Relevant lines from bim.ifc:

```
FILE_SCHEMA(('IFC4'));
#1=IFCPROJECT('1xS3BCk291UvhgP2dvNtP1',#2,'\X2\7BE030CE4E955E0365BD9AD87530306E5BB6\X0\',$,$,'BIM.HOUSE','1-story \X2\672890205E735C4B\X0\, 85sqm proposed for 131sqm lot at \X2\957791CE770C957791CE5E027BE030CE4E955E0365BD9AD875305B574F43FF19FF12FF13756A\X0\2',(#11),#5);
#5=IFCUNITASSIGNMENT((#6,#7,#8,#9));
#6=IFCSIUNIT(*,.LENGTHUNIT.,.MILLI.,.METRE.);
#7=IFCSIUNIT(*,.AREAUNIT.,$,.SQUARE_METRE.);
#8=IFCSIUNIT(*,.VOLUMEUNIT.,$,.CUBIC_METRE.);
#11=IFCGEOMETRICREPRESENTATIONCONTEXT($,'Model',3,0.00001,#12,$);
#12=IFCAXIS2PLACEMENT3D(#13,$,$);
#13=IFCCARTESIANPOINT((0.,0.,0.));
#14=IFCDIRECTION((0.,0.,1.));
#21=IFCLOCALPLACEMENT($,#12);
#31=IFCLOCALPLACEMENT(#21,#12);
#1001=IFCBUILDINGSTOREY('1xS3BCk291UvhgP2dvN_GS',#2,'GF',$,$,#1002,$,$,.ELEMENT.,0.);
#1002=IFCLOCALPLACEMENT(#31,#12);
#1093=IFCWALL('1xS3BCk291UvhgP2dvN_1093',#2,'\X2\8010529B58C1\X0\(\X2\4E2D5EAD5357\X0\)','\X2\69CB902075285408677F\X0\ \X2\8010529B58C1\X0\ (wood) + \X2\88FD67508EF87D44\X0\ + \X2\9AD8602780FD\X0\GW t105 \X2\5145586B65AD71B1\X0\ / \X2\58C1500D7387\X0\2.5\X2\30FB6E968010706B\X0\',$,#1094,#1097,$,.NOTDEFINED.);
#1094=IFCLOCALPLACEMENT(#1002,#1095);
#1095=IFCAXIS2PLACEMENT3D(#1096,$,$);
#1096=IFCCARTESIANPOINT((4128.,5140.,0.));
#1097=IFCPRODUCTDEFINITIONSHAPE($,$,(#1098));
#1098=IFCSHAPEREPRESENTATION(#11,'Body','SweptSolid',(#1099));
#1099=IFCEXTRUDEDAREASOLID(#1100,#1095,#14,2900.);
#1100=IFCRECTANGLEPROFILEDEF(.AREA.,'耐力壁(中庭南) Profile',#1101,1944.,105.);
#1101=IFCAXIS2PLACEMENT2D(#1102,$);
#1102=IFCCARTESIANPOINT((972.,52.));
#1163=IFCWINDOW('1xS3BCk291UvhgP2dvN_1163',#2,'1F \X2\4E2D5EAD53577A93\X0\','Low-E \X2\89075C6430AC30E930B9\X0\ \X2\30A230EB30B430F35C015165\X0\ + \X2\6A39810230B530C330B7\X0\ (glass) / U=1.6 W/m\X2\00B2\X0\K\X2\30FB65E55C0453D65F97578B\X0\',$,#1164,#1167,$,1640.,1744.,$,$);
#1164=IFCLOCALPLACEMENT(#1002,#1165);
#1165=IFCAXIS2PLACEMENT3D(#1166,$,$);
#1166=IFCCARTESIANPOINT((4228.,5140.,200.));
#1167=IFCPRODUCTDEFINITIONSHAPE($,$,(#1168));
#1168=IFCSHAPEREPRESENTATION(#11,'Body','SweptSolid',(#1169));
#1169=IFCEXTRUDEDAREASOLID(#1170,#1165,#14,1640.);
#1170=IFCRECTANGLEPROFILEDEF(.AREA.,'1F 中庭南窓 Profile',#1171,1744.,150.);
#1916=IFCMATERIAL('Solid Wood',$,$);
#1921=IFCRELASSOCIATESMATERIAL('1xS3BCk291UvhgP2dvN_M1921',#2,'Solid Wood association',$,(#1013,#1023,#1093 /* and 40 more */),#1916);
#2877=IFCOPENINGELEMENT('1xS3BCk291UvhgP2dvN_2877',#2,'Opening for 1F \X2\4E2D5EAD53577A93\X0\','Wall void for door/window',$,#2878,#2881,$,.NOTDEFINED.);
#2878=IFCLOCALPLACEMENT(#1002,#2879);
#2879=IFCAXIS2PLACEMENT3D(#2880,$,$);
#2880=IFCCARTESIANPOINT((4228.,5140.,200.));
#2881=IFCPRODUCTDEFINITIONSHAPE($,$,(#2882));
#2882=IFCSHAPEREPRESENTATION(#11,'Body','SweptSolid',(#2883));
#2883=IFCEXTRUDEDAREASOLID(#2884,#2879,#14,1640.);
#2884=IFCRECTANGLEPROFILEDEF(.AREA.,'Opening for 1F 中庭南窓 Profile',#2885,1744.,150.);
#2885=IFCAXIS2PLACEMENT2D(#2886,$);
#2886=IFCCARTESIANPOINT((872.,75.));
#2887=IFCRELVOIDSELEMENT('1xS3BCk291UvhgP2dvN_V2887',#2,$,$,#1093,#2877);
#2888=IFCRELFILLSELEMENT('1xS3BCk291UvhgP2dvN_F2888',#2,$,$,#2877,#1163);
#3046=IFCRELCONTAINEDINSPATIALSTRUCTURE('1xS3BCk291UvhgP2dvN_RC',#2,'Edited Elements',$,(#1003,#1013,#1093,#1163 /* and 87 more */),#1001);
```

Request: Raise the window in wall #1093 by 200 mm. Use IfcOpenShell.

```python
import numpy as np
import ifcopenshell
import ifcopenshell.api.geometry
import ifcopenshell.util.placement
import ifcopenshell.util.unit

model = ifcopenshell.open("bim.ifc")
unit_scale = ifcopenshell.util.unit.calculate_unit_scale(model)

window = model.by_guid("1xS3BCk291UvhgP2dvN_1163")
opening = window.FillsVoids[0].RelatingOpeningElement
dz = 0.2 / unit_scale

shift = np.array([0.0, 0.0, dz])
# The window is not placed relative to its opening, so move both.
for product in (opening, window):
    matrix = ifcopenshell.util.placement.get_local_placement(product.ObjectPlacement)
    matrix[:3, 3] += shift
    ifcopenshell.api.geometry.edit_object_placement(model, product=product, matrix=matrix, is_si=False)

print(f"moved by {dz * unit_scale:+.3f} m")

model.write("bim_edited.ifc")
```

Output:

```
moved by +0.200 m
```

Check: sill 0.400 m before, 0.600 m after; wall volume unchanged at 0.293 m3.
